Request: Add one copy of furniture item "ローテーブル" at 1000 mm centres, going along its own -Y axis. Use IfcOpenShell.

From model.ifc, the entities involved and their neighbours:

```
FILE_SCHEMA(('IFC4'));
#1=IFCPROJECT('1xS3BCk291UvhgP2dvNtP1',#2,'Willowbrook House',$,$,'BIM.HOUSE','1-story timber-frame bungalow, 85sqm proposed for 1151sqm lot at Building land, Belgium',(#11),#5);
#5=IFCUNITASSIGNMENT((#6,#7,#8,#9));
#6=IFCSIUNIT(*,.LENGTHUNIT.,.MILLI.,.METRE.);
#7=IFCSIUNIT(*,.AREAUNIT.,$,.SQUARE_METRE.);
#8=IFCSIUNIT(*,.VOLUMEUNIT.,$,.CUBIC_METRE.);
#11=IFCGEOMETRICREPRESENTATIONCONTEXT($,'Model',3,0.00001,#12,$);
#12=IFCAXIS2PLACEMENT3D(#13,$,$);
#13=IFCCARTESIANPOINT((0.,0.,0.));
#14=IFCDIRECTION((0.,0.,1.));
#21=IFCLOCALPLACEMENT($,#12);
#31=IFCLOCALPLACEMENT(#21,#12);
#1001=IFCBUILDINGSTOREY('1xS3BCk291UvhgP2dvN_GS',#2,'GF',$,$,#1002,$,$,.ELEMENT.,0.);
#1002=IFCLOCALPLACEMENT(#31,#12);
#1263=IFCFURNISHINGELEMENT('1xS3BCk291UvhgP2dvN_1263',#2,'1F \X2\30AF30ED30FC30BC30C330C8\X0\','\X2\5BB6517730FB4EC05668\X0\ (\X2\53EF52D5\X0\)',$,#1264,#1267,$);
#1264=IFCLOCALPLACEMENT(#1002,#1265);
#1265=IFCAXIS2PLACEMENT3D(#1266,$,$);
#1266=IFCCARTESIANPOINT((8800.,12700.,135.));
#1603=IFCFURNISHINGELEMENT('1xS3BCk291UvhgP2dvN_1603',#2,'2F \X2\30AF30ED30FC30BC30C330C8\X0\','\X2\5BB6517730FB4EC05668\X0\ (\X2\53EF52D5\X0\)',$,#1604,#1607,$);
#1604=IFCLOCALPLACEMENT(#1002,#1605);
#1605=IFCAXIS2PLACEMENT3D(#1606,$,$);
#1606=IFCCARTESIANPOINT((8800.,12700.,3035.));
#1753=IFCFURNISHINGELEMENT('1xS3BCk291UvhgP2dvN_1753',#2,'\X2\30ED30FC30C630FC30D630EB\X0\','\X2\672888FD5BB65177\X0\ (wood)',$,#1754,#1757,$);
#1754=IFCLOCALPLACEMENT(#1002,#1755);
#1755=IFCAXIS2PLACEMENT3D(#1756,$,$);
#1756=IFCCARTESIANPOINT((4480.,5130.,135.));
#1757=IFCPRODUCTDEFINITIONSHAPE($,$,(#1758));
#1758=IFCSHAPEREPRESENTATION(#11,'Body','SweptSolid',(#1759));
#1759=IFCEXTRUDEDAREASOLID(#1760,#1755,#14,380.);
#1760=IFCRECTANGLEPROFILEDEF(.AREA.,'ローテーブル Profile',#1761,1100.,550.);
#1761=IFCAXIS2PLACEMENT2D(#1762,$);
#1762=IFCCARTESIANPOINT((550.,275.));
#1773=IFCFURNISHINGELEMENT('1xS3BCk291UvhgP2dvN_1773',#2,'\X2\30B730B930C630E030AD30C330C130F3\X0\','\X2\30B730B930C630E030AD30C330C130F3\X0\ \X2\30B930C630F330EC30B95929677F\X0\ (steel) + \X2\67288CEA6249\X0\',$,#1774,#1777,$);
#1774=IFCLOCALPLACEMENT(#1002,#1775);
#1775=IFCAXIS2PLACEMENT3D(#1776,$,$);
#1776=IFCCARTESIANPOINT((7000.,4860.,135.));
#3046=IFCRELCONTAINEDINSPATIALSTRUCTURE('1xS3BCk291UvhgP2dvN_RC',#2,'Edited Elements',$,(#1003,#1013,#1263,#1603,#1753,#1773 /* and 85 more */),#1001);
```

```python
import ifcopenshell
import ifcopenshell.api.geometry
import ifcopenshell.api.root
import ifcopenshell.util.element
import ifcopenshell.util.placement

model = ifcopenshell.open("model.ifc")


def reuse_history(source, copy):
    """copy_class also copies each property set's owner history, people and application; keep the originals."""
    for rel in copy.IsDefinedBy:
        if rel.is_a("IfcRelDefinesByProperties") and (history := rel.RelatingPropertyDefinition.OwnerHistory):
            rel.RelatingPropertyDefinition.OwnerHistory = source.OwnerHistory
            ifcopenshell.util.element.remove_deep2(model, history)


source = model.by_guid("1xS3BCk291UvhgP2dvN_1753")
base = ifcopenshell.util.placement.get_local_placement(source.ObjectPlacement)
step = -base[:3, 1] * 1000.0

for i in range(1, 2):
    copy = ifcopenshell.api.root.copy_class(model, product=source)
    copy.Representation = ifcopenshell.util.element.copy_deep(
        model, source.Representation, exclude=["IfcGeometricRepresentationContext", "IfcRepresentationMap"]
    )
    reuse_history(source, copy)
    matrix = base.copy()
    matrix[:3, 3] += i * step
    print("added at", matrix[:3, 3].round(3) + 0.0)
    ifcopenshell.api.geometry.edit_object_placement(model, product=copy, matrix=matrix, is_si=False)

model.write("model_rev.ifc")
```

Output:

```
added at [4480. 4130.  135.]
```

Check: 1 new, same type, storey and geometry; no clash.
